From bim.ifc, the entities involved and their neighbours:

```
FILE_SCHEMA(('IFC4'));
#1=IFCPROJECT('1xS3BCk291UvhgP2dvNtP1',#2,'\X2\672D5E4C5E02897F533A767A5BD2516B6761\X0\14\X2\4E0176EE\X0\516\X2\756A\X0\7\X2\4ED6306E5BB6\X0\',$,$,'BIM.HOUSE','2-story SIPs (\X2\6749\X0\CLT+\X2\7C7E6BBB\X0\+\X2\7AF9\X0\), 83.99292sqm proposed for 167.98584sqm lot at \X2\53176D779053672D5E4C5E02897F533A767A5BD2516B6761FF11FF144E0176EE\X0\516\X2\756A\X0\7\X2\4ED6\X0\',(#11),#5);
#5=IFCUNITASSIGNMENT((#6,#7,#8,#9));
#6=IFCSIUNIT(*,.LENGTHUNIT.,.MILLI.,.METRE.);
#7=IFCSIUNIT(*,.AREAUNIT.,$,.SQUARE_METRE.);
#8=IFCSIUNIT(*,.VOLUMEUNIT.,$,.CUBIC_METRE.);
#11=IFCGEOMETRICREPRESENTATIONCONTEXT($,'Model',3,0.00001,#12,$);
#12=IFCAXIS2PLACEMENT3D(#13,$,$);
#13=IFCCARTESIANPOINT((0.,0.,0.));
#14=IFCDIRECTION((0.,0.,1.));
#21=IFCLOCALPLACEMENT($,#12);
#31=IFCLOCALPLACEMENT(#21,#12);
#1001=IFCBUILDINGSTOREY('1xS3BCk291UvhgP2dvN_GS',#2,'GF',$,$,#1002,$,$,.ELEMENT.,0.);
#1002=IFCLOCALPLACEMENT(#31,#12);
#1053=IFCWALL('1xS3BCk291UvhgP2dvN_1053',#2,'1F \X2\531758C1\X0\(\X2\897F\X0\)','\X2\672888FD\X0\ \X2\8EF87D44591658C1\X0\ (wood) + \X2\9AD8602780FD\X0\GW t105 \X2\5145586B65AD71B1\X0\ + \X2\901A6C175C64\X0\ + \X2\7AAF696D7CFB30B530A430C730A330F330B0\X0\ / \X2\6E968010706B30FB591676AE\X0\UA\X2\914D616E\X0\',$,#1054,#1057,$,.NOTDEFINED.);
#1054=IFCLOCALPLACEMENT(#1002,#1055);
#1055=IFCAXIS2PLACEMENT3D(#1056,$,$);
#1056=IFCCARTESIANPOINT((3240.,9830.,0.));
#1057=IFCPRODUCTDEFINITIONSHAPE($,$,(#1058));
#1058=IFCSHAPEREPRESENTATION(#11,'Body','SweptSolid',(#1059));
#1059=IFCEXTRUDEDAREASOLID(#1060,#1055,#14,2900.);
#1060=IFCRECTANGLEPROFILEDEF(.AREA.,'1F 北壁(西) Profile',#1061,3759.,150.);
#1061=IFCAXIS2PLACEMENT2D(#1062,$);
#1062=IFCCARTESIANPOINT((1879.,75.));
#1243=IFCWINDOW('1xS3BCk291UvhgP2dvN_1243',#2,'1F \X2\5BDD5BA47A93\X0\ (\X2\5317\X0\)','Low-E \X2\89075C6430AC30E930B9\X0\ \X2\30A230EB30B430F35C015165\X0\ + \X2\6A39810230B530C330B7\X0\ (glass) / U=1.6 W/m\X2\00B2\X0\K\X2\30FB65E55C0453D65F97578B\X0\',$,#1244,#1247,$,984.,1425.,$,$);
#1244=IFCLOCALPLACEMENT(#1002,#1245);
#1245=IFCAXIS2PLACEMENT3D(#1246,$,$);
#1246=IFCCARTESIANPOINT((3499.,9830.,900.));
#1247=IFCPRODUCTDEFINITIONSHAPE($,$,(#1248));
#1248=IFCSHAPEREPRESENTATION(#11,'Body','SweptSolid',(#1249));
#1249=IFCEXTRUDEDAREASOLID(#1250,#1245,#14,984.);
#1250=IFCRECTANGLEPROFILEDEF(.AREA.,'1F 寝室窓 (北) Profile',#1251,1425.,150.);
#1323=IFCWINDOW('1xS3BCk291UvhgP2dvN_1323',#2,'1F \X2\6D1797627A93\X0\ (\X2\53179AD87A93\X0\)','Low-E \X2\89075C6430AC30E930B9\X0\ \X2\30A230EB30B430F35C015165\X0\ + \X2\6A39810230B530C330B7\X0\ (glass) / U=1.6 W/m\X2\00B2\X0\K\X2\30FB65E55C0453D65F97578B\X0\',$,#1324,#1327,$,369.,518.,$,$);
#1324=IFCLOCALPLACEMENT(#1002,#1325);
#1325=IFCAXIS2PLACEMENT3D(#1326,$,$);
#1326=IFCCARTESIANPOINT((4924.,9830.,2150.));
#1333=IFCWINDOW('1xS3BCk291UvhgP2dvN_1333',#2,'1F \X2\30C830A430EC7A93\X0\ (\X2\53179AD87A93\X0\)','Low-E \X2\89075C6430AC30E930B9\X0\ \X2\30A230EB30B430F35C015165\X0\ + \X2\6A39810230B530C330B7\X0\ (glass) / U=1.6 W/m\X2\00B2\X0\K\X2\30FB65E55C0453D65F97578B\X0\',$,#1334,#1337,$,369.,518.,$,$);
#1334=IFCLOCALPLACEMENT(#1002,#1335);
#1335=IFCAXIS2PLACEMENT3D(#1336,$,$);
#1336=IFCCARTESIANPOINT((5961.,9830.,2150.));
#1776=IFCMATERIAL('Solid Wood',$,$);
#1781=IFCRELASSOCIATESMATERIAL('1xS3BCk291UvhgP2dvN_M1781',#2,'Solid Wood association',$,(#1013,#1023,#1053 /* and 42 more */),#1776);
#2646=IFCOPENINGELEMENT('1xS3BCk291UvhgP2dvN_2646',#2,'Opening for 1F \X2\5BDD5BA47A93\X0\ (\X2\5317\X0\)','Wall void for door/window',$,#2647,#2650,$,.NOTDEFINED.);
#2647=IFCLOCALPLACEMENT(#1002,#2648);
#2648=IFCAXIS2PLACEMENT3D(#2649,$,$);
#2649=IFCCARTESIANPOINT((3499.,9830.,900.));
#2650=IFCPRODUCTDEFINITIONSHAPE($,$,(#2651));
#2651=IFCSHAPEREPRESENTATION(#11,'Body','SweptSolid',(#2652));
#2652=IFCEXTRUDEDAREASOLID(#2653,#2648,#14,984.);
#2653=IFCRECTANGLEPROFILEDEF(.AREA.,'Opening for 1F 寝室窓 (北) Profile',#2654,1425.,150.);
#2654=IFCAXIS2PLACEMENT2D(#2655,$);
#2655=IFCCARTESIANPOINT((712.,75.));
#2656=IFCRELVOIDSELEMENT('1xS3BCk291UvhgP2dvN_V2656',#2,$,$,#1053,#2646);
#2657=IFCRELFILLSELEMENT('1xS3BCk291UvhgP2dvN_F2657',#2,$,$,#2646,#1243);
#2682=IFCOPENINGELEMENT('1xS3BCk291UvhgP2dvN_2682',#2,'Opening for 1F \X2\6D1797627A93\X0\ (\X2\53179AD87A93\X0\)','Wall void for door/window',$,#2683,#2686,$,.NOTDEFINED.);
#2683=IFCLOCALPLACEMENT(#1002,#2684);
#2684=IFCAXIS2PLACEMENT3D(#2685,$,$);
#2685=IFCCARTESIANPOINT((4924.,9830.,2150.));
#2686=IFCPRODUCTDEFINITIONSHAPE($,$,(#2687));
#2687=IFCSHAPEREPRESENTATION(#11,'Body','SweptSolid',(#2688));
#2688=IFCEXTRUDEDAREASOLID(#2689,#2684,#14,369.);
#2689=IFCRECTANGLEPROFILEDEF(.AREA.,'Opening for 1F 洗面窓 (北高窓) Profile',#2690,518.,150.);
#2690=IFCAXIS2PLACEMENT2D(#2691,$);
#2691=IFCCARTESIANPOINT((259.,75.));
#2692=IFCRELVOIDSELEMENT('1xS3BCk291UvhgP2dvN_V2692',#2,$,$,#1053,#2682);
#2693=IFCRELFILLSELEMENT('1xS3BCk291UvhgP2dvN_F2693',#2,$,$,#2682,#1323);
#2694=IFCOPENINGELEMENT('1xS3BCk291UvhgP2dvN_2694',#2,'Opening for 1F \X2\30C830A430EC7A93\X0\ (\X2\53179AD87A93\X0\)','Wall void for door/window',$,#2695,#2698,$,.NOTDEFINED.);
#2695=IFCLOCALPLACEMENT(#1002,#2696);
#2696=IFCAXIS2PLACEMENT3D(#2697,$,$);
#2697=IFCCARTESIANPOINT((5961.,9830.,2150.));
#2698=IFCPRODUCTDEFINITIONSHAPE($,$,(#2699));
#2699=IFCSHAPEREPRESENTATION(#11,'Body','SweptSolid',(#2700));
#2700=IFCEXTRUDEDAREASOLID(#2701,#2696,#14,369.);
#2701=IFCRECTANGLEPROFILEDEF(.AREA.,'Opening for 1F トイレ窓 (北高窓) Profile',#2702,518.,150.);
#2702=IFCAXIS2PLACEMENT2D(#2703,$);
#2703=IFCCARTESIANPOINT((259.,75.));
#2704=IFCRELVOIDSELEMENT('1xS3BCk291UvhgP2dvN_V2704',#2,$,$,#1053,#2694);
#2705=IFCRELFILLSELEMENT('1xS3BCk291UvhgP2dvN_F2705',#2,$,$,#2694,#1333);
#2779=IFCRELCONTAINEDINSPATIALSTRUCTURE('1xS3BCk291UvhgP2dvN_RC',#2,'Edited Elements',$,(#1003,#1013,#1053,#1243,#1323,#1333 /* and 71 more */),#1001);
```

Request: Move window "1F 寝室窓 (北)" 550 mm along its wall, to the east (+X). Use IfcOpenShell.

```python
import ifcopenshell
import ifcopenshell.api.geometry
import ifcopenshell.util.placement
import ifcopenshell.util.unit

model = ifcopenshell.open("bim.ifc")
unit_scale = ifcopenshell.util.unit.calculate_unit_scale(model)

window = model.by_guid("1xS3BCk291UvhgP2dvN_1243")
opening = window.FillsVoids[0].RelatingOpeningElement
wall = opening.VoidsElements[0].RelatingBuildingElement

wall_matrix = ifcopenshell.util.placement.get_local_placement(wall.ObjectPlacement)
shift = wall_matrix[:3, 0] * 0.55 / unit_scale
before = ifcopenshell.util.placement.get_local_placement(window.ObjectPlacement)[:3, 3].copy()

# The window is not placed relative to its opening, so move both.
for product in (opening, window):
    matrix = ifcopenshell.util.placement.get_local_placement(product.ObjectPlacement)
    matrix[:3, 3] += shift
    ifcopenshell.api.geometry.edit_object_placement(model, product=product, matrix=matrix, is_si=False)

after = ifcopenshell.util.placement.get_local_placement(window.ObjectPlacement)[:3, 3]
print("window moved by", (after - before).round(3) + 0.0)

model.write("bim_edited.ifc")
```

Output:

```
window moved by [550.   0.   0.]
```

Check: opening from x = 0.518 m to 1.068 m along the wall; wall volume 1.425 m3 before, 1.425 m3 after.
